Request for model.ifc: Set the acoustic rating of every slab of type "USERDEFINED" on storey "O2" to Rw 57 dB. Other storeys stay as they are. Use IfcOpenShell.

First a look at what the model holds.

```python
import ifcopenshell
import ifcopenshell.util.element

model = ifcopenshell.open("model.ifc")
print(model.schema)
storey = next(s for s in model.by_type("IfcBuildingStorey") if s.Name == "O2")
slabs = [e for e in ifcopenshell.util.element.get_decomposition(storey) if e.is_a("IfcSlab")]
seen = {}
for e in slabs:
    element_type = ifcopenshell.util.element.get_type(e)
    key = (element_type.Name if element_type != e and element_type else None, ifcopenshell.util.element.get_pset(e, "Pset_SlabCommon", "AcousticRating"))
    seen[key] = seen.get(key, 0) + 1
for (name, value), count in sorted(seen.items(), key=str):
    print(count, "x", name, "|", value)
```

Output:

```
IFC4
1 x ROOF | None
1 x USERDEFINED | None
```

```python
import ifcopenshell
import ifcopenshell.api.pset
import ifcopenshell.util.element

model = ifcopenshell.open("model.ifc")

storey = next(s for s in model.by_type("IfcBuildingStorey") if s.Name == "O2")
slabs = [e for e in ifcopenshell.util.element.get_decomposition(storey) if e.is_a("IfcSlab")]

count = 0
for e in slabs:
    element_type = ifcopenshell.util.element.get_type(e)
    if element_type in (None, e) or element_type.Name != "USERDEFINED":
        continue
    # add_pset returns the element's existing set when there is one.
    pset = ifcopenshell.api.pset.add_pset(model, product=e, name="Pset_SlabCommon")
    ifcopenshell.api.pset.edit_pset(model, pset=pset, properties={"AcousticRating": "Rw 57 dB"})
    count += 1

print(count, "slabs updated")

model.write("model-out.ifc")
```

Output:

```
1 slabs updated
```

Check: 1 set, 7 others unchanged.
